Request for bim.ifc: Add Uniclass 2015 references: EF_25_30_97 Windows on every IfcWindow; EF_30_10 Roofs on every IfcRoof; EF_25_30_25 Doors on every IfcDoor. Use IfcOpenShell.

First a look at what the model holds.

```python
import ifcopenshell

model = ifcopenshell.open("bim.ifc")
print(model.schema)
print("classifications:", [c.Name for c in model.by_type("IfcClassification")])
for ifc_class in ("IfcDoor", "IfcRoof", "IfcStair", "IfcWall", "IfcWindow"):
    print(ifc_class, len(model.by_type(ifc_class)))
```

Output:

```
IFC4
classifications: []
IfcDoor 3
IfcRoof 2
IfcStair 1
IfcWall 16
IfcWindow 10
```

```python
import ifcopenshell
import ifcopenshell.api.classification

model = ifcopenshell.open("bim.ifc")

system = ifcopenshell.api.classification.add_classification(model, classification="Uniclass 2015")

codes = {
    "IfcWindow": ("EF_25_30_97", "Windows"),
    "IfcRoof": ("EF_30_10", "Roofs"),
    "IfcDoor": ("EF_25_30_25", "Doors"),
}
for ifc_class, (code, name) in codes.items():
    products = model.by_type(ifc_class)
    ifcopenshell.api.classification.add_reference(
        model, products=products, classification=system, identification=code, name=name
    )
    print(code, len(products))

model.write("bim_updated.ifc")
```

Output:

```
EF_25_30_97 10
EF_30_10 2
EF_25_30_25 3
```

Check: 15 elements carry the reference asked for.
